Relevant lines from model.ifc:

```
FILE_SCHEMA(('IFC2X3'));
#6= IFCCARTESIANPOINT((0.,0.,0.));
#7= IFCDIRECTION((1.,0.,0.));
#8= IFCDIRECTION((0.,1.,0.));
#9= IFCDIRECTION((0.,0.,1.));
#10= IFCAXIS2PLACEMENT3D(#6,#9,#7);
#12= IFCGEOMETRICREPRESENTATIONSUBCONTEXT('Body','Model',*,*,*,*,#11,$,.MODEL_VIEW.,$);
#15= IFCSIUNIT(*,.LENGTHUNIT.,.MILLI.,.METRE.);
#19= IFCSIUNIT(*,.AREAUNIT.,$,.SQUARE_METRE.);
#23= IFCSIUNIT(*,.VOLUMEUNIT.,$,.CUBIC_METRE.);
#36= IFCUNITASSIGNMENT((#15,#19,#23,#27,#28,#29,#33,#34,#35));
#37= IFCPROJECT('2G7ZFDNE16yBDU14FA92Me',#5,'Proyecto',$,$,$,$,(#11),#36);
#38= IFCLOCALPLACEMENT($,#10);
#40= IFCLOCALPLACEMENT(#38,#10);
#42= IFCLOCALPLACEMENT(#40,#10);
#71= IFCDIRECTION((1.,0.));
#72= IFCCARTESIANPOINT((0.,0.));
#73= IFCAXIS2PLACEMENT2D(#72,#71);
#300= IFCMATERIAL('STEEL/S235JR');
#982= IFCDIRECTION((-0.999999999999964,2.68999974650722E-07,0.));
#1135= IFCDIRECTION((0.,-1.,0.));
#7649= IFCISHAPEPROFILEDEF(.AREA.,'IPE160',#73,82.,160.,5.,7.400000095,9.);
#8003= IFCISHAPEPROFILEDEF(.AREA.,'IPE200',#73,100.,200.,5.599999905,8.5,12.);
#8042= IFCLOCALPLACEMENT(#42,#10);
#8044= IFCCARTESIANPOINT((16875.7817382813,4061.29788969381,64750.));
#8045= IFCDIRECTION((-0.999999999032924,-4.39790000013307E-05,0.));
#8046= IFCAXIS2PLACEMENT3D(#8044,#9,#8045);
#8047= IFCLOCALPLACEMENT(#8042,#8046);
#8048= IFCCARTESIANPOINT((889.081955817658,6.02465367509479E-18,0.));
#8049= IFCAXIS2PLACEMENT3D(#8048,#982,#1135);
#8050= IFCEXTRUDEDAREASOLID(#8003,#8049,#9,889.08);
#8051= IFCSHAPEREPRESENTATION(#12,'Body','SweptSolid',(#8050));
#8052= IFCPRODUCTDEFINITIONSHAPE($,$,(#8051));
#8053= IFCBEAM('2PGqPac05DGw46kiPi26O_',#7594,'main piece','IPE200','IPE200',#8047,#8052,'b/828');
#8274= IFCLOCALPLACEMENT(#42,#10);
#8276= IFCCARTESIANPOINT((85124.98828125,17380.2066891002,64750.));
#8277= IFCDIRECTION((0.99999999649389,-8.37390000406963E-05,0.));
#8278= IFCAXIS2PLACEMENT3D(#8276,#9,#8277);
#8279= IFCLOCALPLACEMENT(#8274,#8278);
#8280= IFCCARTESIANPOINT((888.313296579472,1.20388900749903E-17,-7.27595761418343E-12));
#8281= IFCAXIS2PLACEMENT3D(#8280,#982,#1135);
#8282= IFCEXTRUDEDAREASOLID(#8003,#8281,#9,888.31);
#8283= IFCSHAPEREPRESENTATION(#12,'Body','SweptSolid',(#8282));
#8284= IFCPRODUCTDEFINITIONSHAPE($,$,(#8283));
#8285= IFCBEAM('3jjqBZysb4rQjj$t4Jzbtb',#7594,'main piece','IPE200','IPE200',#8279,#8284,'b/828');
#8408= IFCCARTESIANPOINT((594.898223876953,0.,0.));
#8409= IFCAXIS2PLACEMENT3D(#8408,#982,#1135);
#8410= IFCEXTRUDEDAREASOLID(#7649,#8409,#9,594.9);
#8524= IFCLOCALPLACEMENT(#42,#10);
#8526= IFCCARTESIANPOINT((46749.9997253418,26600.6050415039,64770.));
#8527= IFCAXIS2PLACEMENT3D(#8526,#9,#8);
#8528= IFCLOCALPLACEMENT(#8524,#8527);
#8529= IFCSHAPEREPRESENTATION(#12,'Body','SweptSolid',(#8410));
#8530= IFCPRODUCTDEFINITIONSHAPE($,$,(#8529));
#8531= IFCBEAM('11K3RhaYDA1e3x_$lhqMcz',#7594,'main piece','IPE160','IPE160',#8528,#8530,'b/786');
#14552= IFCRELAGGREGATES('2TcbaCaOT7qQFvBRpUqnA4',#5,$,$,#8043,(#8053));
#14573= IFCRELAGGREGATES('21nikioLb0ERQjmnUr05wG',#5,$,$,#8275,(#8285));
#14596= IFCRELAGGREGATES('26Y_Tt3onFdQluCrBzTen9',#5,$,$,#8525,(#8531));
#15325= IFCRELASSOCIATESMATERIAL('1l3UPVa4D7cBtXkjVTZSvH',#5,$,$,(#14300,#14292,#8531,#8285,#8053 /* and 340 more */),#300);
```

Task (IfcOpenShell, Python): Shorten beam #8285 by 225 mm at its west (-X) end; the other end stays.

```python
import ifcopenshell
import ifcopenshell.util.representation
import ifcopenshell.util.unit

model = ifcopenshell.open("model.ifc")
unit_scale = ifcopenshell.util.unit.calculate_unit_scale(model)

member = model.by_id(8285)
change = -0.225 / unit_scale

# The extrusion runs towards the end named, so only its depth changes.
body = ifcopenshell.util.representation.get_representation(member, "Model", "Body")
solid = body.Items[0]
old_length = solid.Depth
solid.Depth += change

print(f"length {old_length:g} -> {solid.Depth:g}")

model.write("model-out.ifc")
```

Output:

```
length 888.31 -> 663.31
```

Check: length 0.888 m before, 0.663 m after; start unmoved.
